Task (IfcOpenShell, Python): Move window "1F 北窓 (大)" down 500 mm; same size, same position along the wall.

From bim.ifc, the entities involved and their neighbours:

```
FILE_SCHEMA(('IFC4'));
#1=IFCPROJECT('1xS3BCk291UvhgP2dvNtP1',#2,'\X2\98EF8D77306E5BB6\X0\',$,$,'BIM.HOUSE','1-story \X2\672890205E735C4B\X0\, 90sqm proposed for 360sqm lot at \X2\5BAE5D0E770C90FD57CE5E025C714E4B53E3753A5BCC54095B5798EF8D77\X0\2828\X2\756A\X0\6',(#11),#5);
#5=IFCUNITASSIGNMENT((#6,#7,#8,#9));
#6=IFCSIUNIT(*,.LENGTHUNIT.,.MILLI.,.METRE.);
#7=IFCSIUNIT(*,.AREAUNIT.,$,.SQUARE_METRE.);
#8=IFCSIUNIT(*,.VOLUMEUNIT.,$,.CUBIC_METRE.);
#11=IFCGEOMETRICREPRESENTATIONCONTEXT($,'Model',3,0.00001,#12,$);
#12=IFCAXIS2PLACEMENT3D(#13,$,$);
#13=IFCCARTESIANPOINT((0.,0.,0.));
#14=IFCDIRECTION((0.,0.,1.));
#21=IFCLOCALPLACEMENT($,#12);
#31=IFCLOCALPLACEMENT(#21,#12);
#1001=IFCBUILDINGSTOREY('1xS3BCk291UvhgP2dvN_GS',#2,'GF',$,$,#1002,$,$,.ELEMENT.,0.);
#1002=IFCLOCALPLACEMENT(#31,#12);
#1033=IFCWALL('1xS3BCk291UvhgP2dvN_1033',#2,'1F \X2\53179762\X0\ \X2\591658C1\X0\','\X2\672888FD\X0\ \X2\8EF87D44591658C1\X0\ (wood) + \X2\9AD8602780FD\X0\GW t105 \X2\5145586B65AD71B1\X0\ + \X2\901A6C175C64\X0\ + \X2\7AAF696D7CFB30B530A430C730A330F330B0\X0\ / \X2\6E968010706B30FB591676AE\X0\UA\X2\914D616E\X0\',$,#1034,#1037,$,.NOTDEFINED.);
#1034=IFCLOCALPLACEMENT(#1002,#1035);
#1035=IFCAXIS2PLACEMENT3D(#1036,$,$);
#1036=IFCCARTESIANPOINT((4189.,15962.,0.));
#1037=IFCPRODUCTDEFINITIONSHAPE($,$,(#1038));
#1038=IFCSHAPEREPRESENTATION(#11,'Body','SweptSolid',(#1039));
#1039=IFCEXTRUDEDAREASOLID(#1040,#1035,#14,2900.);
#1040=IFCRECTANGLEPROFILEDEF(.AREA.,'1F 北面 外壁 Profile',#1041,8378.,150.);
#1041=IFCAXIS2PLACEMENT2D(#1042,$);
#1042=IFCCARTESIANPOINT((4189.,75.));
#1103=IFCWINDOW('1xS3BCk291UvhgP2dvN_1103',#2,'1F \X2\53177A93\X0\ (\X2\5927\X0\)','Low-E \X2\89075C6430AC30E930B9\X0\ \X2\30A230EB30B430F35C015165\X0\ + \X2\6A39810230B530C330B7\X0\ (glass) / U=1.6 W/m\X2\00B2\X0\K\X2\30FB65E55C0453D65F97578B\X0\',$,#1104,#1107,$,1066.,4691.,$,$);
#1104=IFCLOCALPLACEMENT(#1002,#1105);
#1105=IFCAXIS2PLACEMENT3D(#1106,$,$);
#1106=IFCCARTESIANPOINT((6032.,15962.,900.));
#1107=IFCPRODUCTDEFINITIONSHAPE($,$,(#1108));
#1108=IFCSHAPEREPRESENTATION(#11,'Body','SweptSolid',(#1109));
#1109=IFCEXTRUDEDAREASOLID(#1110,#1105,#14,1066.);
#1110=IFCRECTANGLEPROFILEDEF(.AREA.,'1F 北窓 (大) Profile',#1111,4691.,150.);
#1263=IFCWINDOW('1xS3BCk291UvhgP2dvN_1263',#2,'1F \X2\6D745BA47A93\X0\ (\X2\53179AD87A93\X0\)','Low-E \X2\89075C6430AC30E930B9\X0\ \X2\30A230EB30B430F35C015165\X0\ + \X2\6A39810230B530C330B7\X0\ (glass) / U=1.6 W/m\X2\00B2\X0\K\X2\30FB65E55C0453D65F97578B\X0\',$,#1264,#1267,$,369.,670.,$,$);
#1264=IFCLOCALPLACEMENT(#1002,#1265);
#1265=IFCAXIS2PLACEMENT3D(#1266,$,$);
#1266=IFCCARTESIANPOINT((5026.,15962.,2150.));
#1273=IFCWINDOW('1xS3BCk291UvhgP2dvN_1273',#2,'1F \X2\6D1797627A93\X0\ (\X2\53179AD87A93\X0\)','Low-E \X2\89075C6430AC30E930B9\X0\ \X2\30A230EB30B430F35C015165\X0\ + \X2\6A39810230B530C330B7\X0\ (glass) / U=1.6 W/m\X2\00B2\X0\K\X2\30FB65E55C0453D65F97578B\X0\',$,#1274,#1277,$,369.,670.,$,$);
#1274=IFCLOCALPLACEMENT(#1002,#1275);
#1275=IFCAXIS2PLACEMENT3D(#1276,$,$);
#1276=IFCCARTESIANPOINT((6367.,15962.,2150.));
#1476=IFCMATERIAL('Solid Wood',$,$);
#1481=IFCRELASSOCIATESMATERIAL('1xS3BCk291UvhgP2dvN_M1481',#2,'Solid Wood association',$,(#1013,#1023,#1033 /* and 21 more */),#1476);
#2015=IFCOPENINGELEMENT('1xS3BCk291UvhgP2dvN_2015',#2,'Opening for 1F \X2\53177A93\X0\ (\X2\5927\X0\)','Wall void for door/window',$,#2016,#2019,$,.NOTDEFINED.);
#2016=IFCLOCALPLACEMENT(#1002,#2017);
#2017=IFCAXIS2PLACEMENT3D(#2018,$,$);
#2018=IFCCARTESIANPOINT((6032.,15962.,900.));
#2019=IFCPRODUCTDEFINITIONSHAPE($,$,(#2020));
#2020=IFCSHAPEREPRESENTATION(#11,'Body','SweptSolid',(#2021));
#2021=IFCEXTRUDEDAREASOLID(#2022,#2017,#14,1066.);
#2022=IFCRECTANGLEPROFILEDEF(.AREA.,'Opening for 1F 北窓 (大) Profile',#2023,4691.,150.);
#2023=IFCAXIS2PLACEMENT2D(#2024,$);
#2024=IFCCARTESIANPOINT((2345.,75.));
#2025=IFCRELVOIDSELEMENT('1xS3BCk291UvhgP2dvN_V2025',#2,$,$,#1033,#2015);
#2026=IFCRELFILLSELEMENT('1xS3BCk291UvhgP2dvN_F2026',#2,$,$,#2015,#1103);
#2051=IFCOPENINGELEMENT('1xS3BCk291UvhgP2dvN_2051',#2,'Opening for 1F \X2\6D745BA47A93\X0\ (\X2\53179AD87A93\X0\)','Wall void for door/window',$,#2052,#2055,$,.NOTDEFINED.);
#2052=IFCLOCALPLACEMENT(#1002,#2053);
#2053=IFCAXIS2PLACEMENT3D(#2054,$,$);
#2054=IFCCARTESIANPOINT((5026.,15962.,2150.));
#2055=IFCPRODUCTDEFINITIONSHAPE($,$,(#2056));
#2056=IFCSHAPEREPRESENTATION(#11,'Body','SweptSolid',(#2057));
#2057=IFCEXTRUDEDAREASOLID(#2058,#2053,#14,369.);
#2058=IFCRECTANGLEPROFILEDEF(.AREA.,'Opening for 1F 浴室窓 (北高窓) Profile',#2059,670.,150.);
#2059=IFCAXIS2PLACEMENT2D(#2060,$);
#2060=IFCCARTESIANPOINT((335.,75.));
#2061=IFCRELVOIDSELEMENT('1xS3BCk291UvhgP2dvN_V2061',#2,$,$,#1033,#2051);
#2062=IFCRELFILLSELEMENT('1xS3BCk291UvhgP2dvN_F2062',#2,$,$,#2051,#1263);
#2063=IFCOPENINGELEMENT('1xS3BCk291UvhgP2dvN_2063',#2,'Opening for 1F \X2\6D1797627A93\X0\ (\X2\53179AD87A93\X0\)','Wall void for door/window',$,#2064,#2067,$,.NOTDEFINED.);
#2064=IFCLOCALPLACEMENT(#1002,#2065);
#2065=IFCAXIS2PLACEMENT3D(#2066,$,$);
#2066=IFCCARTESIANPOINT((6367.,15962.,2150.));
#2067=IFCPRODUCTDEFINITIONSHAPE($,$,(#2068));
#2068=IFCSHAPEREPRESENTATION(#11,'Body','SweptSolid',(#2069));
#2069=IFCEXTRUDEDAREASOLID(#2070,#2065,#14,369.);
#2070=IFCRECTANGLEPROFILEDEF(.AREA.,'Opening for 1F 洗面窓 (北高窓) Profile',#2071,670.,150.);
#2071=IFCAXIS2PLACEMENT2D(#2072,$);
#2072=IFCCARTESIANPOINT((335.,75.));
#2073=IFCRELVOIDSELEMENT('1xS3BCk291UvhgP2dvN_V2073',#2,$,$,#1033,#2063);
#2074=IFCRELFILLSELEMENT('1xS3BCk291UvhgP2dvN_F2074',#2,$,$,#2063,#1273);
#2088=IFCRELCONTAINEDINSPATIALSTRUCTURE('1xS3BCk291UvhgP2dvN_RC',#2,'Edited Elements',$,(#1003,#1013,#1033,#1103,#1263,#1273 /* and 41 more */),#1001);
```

```python
import numpy as np
import ifcopenshell
import ifcopenshell.api.geometry
import ifcopenshell.util.placement
import ifcopenshell.util.unit

model = ifcopenshell.open("bim.ifc")
unit_scale = ifcopenshell.util.unit.calculate_unit_scale(model)

window = model.by_guid("1xS3BCk291UvhgP2dvN_1103")
opening = window.FillsVoids[0].RelatingOpeningElement
dz = -0.5 / unit_scale

shift = np.array([0.0, 0.0, dz])
# The window is not placed relative to its opening, so move both.
for product in (opening, window):
    matrix = ifcopenshell.util.placement.get_local_placement(product.ObjectPlacement)
    matrix[:3, 3] += shift
    ifcopenshell.api.geometry.edit_object_placement(model, product=product, matrix=matrix, is_si=False)

print(f"moved by {dz * unit_scale:+.3f} m")

model.write("bim_edited.ifc")
```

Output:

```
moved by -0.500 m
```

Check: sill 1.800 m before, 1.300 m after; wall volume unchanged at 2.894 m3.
